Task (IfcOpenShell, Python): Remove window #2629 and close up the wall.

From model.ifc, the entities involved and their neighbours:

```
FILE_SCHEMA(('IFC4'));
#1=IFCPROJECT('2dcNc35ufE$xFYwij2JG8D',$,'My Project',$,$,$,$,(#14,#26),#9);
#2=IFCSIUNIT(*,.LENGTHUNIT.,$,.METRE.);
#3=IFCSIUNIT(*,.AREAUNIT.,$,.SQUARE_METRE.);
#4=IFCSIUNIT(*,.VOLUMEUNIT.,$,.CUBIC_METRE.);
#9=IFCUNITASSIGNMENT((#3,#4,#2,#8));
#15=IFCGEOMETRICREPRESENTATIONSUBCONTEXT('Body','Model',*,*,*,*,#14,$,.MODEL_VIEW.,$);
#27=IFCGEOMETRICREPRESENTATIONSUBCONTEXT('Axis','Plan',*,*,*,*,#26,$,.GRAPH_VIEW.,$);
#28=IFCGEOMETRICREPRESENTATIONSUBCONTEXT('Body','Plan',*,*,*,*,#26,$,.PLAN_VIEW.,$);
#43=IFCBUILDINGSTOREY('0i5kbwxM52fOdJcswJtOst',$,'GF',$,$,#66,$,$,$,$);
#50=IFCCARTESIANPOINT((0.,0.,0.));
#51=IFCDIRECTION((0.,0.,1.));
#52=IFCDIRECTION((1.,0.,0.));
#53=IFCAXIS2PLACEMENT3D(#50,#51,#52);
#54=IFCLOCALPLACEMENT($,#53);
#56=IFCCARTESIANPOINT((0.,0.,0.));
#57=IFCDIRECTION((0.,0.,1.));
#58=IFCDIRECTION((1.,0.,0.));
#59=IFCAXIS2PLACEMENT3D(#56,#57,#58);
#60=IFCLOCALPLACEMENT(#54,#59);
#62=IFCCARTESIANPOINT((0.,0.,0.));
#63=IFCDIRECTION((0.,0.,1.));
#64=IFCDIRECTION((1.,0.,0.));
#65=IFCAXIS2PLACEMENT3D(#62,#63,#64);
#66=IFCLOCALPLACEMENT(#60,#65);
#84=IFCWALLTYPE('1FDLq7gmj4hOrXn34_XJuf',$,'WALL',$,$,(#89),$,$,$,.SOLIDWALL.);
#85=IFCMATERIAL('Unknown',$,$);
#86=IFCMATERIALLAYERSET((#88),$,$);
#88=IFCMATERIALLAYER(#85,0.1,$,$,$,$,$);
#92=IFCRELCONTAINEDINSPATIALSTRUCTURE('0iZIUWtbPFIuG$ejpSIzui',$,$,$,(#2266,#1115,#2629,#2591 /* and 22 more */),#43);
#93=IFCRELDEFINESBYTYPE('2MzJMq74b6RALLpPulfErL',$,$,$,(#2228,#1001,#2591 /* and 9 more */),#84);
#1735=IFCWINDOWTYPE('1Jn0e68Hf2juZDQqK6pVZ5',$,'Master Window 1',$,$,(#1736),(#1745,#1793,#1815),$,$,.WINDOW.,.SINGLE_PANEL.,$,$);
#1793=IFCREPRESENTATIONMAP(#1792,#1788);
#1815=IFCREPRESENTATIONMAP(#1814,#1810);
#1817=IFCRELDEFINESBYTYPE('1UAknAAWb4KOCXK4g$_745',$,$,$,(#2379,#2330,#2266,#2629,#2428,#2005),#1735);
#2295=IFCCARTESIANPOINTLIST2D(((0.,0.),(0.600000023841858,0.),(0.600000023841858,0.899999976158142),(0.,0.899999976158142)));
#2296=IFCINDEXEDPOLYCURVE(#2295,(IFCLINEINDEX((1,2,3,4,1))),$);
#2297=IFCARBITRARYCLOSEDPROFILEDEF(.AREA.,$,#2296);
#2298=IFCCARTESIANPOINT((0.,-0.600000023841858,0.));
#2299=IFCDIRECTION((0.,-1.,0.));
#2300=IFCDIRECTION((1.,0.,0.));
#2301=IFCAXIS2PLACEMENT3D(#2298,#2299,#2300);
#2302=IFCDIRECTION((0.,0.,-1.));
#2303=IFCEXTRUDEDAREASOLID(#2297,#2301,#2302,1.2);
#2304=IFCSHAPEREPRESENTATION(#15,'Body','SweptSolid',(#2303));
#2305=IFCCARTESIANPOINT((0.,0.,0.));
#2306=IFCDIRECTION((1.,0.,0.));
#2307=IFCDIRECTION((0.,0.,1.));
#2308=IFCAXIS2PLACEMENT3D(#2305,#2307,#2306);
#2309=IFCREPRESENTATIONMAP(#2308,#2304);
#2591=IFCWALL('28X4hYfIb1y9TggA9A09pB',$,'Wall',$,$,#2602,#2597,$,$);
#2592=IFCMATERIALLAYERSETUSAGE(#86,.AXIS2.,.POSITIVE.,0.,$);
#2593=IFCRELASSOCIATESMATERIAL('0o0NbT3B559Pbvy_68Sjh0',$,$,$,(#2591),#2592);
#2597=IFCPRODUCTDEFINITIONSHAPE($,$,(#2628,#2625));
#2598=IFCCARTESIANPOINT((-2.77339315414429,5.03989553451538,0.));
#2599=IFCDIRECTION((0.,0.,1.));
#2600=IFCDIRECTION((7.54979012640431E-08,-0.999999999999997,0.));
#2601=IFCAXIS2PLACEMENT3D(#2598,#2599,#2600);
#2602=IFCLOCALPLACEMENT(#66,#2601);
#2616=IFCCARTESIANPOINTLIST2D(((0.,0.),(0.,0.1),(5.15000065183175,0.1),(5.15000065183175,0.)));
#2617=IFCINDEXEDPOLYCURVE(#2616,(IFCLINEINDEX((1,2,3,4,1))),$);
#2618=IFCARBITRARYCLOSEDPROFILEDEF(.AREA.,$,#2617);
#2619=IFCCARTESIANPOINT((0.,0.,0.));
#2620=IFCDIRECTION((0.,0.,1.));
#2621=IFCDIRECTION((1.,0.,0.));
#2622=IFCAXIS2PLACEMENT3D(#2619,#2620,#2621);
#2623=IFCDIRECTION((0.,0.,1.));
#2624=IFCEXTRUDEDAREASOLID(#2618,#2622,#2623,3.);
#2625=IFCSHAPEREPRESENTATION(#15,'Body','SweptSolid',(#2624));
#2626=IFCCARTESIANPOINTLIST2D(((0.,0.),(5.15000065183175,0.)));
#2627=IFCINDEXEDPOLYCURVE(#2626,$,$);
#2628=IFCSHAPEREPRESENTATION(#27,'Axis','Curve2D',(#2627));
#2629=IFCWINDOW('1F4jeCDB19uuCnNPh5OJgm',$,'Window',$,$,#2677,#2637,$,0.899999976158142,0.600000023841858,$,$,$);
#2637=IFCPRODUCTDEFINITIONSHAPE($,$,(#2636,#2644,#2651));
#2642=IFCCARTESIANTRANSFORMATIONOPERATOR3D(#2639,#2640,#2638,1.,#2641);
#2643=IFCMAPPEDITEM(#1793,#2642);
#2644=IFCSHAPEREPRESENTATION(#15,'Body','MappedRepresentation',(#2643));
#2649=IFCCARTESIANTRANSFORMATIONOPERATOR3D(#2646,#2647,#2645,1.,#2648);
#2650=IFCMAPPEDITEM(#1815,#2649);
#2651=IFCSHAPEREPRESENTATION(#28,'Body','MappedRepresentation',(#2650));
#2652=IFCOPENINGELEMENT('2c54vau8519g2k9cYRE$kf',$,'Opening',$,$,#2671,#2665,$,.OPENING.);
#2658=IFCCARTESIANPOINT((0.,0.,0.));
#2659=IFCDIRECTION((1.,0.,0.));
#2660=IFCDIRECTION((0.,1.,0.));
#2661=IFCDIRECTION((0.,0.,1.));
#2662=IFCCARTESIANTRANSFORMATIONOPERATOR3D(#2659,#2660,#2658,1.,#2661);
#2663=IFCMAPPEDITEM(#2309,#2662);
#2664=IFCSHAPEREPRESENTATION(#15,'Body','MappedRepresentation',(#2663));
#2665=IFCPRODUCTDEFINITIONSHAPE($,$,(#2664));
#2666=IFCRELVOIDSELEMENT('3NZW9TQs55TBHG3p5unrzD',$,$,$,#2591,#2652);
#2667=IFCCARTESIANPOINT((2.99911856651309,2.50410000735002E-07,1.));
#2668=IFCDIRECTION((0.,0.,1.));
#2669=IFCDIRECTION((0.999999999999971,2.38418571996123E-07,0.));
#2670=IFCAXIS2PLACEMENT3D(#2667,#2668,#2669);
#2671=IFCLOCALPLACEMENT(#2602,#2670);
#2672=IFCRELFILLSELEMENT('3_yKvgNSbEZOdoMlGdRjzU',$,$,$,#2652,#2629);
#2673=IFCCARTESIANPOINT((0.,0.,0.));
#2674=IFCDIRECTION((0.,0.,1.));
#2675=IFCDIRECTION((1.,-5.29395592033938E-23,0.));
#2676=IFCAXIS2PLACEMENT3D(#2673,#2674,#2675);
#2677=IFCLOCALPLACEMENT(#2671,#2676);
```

```python
import ifcopenshell
import ifcopenshell.api.feature
import ifcopenshell.api.root
import ifcopenshell.geom
import ifcopenshell.util.shape

model = ifcopenshell.open("model.ifc")
settings = ifcopenshell.geom.settings()


def volume(element):
    """Net volume in cubic metres, openings subtracted."""
    shape = ifcopenshell.geom.create_shape(settings, element)
    return ifcopenshell.util.shape.get_volume(shape.geometry)


window = model.by_guid("1F4jeCDB19uuCnNPh5OJgm")
opening = window.FillsVoids[0].RelatingOpeningElement
wall = opening.VoidsElements[0].RelatingBuildingElement
before = volume(wall)

ifcopenshell.api.root.remove_product(model, product=window)
ifcopenshell.api.feature.remove_feature(model, feature=opening)

after = volume(wall)

print(f"wall volume {before:.3f} -> {after:.3f} m3")

model.write("model_edited.ifc")
```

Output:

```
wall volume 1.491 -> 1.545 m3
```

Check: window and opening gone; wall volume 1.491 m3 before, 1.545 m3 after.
